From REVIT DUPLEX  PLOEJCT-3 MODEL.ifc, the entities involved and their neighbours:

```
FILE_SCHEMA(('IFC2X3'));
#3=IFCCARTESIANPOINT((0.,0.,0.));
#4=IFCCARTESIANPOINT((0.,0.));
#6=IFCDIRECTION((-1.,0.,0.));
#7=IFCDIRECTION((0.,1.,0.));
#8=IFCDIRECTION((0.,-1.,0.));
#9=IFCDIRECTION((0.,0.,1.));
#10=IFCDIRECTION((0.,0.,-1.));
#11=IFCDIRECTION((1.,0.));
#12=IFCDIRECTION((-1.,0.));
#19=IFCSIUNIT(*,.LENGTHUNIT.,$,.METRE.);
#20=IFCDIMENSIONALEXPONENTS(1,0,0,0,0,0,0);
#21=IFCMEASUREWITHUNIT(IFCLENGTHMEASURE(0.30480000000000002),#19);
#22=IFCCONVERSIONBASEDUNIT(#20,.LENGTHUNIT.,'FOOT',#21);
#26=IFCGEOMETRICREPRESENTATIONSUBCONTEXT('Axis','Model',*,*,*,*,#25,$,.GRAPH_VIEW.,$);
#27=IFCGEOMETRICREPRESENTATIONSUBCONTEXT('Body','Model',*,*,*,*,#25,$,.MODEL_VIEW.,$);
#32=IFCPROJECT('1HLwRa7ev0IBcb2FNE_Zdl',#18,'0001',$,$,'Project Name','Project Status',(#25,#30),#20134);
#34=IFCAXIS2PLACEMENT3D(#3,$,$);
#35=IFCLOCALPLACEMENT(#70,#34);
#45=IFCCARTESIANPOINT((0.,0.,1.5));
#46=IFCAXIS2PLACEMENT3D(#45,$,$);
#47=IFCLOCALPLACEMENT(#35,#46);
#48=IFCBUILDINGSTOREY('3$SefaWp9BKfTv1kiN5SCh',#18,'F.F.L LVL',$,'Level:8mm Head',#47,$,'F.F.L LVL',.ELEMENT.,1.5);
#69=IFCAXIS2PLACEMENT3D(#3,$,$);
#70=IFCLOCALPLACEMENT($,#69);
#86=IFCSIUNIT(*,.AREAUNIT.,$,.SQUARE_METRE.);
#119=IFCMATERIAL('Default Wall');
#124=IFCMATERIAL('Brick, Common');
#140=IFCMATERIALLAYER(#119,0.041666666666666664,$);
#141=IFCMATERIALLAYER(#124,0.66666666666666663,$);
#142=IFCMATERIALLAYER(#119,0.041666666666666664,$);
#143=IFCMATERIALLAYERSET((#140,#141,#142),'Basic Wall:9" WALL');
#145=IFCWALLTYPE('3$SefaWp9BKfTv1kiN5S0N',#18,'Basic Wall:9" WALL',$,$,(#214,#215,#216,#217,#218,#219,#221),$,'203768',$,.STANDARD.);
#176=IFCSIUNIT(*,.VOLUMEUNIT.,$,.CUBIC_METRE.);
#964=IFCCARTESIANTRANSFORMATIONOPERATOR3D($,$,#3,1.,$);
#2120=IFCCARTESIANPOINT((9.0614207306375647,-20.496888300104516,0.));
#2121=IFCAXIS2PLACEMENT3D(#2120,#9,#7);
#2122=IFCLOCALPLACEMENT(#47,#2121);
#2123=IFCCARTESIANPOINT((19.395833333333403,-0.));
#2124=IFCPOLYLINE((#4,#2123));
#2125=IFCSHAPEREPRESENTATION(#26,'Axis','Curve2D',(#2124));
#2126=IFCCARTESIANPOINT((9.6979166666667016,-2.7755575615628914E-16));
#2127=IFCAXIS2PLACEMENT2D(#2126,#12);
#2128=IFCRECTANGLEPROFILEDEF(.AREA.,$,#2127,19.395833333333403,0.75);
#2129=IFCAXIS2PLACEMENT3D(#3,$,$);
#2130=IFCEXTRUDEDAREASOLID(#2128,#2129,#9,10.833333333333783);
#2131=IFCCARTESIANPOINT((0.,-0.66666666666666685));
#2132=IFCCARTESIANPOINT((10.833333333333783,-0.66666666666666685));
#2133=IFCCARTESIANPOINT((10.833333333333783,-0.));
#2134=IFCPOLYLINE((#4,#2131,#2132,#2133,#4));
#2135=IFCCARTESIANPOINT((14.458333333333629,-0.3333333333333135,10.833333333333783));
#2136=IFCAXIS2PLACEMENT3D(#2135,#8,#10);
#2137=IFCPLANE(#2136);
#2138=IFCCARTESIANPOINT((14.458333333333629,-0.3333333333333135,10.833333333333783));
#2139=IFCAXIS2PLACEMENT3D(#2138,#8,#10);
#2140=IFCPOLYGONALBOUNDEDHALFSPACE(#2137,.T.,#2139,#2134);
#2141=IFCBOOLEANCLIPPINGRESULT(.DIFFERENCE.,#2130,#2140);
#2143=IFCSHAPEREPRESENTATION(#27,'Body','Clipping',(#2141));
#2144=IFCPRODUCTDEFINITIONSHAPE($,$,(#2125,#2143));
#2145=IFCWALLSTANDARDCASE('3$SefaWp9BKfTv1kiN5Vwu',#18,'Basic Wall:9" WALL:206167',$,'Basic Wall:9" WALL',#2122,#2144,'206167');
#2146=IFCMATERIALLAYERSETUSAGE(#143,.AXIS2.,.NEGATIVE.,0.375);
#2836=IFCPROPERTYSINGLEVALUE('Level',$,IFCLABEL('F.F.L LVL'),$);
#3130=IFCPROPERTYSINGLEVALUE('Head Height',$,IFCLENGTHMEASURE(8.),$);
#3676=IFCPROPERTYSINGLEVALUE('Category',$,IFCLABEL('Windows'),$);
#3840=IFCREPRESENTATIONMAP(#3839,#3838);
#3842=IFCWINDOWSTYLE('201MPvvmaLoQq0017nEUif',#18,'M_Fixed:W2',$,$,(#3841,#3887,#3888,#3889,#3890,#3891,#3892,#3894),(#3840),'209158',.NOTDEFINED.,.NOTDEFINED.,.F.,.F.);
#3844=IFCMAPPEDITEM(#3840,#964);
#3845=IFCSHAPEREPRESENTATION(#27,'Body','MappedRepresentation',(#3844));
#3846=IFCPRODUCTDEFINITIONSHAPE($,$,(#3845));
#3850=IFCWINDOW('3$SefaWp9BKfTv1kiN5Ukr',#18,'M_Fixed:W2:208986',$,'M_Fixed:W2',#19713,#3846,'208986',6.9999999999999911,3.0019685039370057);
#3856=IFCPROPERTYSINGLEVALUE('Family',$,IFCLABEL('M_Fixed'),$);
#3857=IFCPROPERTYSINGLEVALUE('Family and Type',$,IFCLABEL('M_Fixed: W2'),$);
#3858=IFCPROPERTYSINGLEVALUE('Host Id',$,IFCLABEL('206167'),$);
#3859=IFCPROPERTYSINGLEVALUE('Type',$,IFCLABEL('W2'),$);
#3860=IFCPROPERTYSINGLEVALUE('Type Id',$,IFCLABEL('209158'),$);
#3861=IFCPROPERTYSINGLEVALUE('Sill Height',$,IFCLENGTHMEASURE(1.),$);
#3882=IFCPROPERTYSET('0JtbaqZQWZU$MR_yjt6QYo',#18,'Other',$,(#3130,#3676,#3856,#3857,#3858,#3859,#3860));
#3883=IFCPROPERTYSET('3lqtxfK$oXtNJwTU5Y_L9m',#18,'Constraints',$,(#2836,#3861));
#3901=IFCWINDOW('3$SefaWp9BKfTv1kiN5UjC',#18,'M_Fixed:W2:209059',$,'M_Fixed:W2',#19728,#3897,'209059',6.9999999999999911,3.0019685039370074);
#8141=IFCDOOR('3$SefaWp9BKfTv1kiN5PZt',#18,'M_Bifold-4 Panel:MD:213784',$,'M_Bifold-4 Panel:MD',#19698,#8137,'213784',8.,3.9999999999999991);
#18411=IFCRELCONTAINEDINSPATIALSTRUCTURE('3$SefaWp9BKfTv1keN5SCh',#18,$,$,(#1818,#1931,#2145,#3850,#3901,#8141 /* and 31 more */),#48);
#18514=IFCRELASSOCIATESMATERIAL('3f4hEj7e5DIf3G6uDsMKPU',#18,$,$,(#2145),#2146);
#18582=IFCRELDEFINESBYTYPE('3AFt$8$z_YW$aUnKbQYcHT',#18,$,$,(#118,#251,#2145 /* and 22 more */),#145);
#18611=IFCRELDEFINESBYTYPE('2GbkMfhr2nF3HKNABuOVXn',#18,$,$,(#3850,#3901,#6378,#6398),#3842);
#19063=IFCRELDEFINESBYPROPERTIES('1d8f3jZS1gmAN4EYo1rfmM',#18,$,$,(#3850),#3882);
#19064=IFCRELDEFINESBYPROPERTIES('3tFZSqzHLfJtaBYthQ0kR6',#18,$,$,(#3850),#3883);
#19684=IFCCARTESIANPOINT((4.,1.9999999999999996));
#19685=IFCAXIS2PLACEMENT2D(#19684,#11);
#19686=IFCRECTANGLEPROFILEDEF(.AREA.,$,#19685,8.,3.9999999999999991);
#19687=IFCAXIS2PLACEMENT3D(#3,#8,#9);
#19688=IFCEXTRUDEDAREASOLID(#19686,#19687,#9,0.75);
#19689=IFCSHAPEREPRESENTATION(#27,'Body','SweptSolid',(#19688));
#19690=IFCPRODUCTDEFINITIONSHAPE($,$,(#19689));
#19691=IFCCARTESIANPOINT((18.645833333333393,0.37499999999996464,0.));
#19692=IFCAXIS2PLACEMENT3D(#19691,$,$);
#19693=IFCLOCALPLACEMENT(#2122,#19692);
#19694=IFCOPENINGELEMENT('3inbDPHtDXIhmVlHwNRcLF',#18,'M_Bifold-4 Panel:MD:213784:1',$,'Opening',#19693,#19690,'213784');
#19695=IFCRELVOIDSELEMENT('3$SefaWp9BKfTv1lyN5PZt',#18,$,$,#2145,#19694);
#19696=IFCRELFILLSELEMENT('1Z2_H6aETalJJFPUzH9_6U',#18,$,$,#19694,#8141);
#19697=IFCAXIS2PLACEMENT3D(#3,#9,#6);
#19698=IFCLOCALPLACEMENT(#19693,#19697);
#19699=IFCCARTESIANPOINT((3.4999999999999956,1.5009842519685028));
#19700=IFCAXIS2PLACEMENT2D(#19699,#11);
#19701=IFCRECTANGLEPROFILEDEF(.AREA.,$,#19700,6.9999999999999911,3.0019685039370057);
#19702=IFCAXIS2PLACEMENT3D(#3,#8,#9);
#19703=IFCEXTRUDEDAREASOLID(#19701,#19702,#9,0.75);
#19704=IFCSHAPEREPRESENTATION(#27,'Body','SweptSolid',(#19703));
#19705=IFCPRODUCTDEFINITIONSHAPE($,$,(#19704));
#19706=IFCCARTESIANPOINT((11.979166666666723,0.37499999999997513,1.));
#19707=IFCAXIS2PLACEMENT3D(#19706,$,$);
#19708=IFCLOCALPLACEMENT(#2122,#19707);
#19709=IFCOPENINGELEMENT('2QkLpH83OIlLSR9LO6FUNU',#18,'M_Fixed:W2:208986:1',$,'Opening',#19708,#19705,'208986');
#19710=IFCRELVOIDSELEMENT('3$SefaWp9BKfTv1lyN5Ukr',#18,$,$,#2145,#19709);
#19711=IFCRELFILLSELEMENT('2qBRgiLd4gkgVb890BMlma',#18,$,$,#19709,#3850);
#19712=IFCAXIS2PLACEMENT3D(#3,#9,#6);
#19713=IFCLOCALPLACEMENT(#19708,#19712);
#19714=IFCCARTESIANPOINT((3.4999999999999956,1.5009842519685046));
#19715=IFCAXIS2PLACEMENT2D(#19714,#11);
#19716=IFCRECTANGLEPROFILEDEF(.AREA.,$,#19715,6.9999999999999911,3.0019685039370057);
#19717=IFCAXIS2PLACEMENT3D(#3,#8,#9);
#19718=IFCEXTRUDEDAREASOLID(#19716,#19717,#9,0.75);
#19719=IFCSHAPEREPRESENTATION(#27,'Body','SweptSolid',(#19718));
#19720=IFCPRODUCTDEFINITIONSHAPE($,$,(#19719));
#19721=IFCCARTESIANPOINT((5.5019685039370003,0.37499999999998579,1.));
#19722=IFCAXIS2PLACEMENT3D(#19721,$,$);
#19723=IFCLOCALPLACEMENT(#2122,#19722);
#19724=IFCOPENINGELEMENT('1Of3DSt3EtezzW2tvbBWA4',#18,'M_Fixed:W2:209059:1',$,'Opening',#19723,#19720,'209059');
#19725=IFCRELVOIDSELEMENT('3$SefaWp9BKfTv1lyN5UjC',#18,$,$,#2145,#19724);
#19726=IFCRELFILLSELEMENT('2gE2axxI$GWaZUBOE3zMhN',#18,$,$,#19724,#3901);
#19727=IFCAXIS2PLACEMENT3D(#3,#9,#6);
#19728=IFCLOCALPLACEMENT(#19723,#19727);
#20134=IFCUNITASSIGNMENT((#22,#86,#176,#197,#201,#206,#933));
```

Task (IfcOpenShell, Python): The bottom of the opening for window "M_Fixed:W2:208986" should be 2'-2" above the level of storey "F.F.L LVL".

```python
import numpy as np
import ifcopenshell
import ifcopenshell.api.geometry
import ifcopenshell.api.pset
import ifcopenshell.geom
import ifcopenshell.util.element
import ifcopenshell.util.placement
import ifcopenshell.util.shape
import ifcopenshell.util.unit

model = ifcopenshell.open("REVIT DUPLEX  PLOEJCT-3 MODEL.ifc")
unit_scale = ifcopenshell.util.unit.calculate_unit_scale(model)

window = model.by_guid("3$SefaWp9BKfTv1kiN5Ukr")
opening = window.FillsVoids[0].RelatingOpeningElement
storey = ifcopenshell.util.element.get_container(window, ifc_class="IfcBuildingStorey")
level = ifcopenshell.util.placement.get_local_placement(storey.ObjectPlacement)[2, 3]

# The opening's origin need not be at the sill, so measure its lowest point.
shape = ifcopenshell.geom.create_shape(ifcopenshell.geom.settings(), opening)
bottom = ifcopenshell.util.shape.get_shape_bottom_elevation(shape, shape.geometry) / unit_scale
dz = level + 26 * 0.0254 / unit_scale - bottom

shift = np.array([0.0, 0.0, dz])
# The window is placed relative to its opening, so it follows when the opening moves.
matrix = ifcopenshell.util.placement.get_local_placement(opening.ObjectPlacement)
matrix[:3, 3] += shift
ifcopenshell.api.geometry.edit_object_placement(
    model, product=opening, matrix=matrix, is_si=False, should_transform_children=True
)

# Keep the stored heights in step.
pset = model.by_id(ifcopenshell.util.element.get_pset(window, "Other", should_inherit=False)["id"])
ifcopenshell.api.pset.edit_pset(model, pset=pset, properties={
    "Head Height": model.create_entity("IfcLengthMeasure", ifcopenshell.util.element.get_pset(window, "Other", "Head Height") + dz),
})
pset = model.by_id(ifcopenshell.util.element.get_pset(window, "Constraints", should_inherit=False)["id"])
ifcopenshell.api.pset.edit_pset(model, pset=pset, properties={
    "Sill Height": model.create_entity("IfcLengthMeasure", ifcopenshell.util.element.get_pset(window, "Constraints", "Sill Height") + dz),
})

print(f"moved by {dz * unit_scale:+.3f} m")

model.write("REVIT DUPLEX  PLOEJCT-3 MODEL_v2.ifc")
```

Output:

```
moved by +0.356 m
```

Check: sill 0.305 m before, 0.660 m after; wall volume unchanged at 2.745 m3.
